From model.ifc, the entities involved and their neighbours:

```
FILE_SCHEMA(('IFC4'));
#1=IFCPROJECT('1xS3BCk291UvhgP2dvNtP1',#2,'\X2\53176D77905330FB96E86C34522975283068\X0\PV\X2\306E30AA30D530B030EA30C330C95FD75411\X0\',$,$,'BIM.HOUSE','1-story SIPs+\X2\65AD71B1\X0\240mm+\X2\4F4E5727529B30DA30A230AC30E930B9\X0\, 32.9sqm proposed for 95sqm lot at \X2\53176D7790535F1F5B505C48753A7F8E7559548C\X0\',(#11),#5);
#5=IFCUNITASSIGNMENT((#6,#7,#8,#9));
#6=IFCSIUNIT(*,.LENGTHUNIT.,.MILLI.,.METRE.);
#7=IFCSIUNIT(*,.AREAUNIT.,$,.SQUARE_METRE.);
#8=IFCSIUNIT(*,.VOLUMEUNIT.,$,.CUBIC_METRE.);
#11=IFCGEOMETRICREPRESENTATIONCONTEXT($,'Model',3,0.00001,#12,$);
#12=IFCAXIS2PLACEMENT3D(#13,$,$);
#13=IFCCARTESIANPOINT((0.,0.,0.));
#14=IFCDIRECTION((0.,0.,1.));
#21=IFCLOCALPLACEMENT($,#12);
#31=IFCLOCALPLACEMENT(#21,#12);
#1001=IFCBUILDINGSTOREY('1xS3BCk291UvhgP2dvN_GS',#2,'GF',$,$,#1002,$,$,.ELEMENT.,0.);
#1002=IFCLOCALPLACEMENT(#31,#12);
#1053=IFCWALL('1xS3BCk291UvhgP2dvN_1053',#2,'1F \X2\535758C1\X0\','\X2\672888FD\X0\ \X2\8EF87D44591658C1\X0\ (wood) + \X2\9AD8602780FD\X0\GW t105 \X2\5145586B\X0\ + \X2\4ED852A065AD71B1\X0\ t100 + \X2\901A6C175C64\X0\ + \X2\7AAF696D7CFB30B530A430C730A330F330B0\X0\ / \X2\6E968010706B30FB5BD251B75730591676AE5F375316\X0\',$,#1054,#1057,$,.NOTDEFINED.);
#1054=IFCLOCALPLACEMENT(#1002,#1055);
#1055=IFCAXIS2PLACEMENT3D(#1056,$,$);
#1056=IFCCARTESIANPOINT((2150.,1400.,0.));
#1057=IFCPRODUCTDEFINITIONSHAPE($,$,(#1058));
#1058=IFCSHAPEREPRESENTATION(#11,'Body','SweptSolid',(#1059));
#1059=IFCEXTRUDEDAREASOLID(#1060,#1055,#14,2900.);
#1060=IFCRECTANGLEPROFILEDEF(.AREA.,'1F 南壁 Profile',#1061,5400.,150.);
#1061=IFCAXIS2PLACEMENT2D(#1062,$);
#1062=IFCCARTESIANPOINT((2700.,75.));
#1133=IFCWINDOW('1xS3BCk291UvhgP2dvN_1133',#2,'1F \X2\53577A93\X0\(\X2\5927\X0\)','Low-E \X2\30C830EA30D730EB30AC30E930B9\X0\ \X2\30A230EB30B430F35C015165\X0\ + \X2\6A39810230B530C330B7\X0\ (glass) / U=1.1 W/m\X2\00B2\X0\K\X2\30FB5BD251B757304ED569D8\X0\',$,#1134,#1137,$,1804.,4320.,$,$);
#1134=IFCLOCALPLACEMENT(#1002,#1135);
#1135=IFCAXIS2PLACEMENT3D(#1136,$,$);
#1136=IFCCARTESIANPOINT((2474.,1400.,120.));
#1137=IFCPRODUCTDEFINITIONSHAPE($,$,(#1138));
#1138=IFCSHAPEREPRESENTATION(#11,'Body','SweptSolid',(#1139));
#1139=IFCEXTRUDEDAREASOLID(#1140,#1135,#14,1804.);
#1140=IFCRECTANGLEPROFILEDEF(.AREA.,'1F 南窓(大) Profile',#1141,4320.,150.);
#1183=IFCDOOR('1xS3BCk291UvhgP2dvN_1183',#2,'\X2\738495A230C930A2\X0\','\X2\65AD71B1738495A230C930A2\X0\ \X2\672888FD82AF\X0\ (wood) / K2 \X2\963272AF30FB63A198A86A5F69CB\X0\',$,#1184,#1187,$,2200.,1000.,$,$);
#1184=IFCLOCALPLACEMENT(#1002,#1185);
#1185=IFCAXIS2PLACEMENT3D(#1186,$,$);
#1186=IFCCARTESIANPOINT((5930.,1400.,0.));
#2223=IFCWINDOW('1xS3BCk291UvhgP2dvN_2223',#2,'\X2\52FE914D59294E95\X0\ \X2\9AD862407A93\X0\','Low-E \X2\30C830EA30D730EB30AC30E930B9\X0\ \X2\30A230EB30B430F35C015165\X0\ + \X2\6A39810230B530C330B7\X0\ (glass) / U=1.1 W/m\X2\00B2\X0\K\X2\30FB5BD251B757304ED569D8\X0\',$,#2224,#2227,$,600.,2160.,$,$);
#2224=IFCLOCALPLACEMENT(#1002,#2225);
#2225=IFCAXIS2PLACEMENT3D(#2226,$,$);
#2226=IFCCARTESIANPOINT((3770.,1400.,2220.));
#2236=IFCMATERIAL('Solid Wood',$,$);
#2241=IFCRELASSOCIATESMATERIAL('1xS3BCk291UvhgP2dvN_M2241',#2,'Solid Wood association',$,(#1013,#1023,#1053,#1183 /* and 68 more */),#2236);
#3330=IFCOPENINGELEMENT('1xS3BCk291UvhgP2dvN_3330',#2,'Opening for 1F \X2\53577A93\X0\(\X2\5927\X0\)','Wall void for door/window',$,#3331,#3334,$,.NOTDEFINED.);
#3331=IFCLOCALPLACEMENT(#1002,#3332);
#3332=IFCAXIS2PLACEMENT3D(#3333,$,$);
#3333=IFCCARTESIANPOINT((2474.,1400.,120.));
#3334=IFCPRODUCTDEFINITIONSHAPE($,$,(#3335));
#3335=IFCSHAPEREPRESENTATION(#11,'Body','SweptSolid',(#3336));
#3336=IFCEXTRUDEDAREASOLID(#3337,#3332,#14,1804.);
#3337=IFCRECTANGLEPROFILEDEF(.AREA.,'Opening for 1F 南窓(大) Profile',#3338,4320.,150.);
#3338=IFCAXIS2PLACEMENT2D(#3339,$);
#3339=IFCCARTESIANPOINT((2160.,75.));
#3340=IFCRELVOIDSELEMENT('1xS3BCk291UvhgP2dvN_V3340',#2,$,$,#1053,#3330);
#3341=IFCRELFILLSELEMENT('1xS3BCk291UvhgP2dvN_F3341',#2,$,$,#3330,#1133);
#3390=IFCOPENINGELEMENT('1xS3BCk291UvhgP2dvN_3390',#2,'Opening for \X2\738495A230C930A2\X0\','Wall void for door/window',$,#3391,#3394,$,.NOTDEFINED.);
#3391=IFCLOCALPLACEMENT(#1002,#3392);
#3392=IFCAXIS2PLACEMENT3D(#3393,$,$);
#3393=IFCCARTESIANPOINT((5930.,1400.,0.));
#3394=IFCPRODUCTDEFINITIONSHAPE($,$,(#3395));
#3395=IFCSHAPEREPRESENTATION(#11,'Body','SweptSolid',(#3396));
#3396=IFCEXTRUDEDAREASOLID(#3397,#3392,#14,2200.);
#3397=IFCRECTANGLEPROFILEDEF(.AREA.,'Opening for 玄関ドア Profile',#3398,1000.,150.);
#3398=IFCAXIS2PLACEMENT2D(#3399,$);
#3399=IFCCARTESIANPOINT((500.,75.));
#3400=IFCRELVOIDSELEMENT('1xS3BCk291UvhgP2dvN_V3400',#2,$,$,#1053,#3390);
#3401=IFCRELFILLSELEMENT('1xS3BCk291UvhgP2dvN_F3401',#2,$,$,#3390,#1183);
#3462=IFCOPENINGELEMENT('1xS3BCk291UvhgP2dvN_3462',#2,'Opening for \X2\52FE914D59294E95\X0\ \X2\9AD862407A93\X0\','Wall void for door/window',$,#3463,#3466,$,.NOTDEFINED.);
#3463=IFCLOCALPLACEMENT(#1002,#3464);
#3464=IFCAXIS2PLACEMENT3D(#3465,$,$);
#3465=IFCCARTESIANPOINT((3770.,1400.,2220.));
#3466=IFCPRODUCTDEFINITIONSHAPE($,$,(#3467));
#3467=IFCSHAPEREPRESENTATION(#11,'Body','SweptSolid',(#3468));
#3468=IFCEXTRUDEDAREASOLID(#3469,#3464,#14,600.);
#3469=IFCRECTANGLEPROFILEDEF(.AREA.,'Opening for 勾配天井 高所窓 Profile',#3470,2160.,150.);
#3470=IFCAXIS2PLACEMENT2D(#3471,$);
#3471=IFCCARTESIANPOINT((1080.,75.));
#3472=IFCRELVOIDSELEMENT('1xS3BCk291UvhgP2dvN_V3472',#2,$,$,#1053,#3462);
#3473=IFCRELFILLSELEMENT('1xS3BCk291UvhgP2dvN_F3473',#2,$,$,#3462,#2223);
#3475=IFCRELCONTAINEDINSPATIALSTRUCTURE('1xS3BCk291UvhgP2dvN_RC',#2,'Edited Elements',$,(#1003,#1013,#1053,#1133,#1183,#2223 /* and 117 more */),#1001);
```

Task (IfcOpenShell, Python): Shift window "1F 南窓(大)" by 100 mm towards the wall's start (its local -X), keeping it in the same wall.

```python
import ifcopenshell
import ifcopenshell.api.geometry
import ifcopenshell.util.placement
import ifcopenshell.util.unit

model = ifcopenshell.open("model.ifc")
unit_scale = ifcopenshell.util.unit.calculate_unit_scale(model)

window = model.by_guid("1xS3BCk291UvhgP2dvN_1133")
opening = window.FillsVoids[0].RelatingOpeningElement
wall = opening.VoidsElements[0].RelatingBuildingElement

wall_matrix = ifcopenshell.util.placement.get_local_placement(wall.ObjectPlacement)
shift = wall_matrix[:3, 0] * -0.1 / unit_scale
before = ifcopenshell.util.placement.get_local_placement(window.ObjectPlacement)[:3, 3].copy()

# The window is not placed relative to its opening, so move both.
for product in (opening, window):
    matrix = ifcopenshell.util.placement.get_local_placement(product.ObjectPlacement)
    matrix[:3, 3] += shift
    ifcopenshell.api.geometry.edit_object_placement(model, product=product, matrix=matrix, is_si=False)

after = ifcopenshell.util.placement.get_local_placement(window.ObjectPlacement)[:3, 3]
print("window moved by", (after - before).round(3) + 0.0)

model.write("model_rev.ifc")
```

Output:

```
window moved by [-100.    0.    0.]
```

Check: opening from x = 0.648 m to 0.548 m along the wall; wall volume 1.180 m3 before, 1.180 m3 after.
